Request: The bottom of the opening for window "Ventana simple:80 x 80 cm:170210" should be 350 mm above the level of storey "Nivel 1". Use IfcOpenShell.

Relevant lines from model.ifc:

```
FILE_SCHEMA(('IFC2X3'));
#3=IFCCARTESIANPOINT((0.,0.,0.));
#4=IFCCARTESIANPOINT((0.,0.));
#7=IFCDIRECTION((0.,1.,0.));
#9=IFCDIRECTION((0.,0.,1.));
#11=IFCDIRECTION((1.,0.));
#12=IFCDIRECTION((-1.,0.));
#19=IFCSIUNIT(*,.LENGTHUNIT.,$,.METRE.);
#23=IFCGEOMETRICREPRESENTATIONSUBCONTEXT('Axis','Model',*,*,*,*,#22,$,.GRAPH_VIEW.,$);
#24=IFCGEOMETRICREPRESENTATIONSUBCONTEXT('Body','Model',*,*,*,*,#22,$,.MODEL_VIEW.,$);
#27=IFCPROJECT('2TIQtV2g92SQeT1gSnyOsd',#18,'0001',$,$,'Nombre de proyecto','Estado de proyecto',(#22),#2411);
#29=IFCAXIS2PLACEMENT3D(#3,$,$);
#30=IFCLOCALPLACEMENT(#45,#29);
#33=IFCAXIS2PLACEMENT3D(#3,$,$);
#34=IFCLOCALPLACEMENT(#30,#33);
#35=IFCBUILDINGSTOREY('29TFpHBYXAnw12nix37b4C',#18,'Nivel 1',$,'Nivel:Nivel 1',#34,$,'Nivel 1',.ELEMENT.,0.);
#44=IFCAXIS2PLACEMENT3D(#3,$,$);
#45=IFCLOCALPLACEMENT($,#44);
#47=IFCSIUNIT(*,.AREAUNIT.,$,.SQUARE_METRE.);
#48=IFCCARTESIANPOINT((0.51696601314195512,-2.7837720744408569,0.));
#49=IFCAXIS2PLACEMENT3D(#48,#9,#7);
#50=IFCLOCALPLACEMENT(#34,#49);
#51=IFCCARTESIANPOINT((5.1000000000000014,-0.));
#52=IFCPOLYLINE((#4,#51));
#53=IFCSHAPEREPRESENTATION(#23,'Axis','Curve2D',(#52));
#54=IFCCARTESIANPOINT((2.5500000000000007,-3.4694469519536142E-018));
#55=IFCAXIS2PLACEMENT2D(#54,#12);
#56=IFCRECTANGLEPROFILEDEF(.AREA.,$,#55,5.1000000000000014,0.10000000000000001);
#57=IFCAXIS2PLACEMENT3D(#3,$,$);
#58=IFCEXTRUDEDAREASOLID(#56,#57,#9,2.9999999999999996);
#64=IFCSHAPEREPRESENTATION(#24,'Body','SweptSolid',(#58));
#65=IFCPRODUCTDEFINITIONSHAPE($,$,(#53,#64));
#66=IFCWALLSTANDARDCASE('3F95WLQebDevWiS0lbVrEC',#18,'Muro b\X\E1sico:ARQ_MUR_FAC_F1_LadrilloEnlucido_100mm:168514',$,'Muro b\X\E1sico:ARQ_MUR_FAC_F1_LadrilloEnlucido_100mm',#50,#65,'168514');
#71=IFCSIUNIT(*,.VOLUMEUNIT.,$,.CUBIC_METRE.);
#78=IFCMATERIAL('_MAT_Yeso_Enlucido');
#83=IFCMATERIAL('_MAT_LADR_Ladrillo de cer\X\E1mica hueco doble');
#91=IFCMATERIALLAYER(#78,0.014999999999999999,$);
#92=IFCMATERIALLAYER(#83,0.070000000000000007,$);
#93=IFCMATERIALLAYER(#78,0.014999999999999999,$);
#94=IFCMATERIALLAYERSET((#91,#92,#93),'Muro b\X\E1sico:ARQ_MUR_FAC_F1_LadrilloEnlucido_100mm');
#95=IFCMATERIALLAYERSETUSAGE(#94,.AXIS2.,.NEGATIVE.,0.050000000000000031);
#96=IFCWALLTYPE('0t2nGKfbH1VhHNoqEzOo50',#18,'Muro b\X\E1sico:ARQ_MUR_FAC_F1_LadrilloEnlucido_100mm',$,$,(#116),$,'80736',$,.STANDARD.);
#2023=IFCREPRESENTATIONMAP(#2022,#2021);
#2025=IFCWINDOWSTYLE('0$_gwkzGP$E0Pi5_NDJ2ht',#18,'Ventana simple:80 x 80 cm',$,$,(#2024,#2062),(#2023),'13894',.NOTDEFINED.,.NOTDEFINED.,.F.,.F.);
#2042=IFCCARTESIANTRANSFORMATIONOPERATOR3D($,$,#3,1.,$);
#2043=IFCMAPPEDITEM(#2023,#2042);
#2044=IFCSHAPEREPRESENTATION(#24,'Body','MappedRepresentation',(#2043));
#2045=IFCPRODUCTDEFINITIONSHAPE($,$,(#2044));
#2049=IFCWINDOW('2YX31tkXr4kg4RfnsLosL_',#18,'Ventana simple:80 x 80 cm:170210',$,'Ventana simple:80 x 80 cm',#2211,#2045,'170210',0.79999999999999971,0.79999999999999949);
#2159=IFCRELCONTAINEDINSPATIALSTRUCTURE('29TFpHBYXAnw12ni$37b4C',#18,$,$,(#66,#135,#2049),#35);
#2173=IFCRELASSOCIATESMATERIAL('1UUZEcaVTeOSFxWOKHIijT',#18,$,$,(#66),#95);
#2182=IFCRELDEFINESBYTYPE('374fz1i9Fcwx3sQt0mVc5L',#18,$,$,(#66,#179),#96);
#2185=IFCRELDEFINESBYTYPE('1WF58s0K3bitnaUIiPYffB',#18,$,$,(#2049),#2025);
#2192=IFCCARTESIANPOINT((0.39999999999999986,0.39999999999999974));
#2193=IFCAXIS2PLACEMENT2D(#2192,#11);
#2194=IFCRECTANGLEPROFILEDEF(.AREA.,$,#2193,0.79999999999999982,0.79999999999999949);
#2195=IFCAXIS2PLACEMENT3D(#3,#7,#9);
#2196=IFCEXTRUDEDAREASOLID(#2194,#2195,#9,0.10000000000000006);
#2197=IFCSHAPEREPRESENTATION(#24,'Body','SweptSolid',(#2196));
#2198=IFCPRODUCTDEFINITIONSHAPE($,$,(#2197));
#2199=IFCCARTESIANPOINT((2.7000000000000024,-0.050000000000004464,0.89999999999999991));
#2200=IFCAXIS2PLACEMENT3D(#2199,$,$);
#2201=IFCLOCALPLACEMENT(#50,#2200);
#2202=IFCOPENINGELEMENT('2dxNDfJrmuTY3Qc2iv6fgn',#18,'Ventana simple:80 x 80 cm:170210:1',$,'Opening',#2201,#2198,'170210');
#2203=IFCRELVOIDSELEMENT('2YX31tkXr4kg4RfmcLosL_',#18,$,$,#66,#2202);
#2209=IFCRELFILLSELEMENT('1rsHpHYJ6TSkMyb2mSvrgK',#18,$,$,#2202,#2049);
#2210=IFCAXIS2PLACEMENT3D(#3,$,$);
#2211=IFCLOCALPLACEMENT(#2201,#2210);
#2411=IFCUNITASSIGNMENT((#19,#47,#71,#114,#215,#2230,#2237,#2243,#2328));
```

```python
import numpy as np
import ifcopenshell
import ifcopenshell.api.geometry
import ifcopenshell.geom
import ifcopenshell.util.element
import ifcopenshell.util.placement
import ifcopenshell.util.shape
import ifcopenshell.util.unit

model = ifcopenshell.open("model.ifc")
unit_scale = ifcopenshell.util.unit.calculate_unit_scale(model)

window = model.by_guid("2YX31tkXr4kg4RfnsLosL_")
opening = window.FillsVoids[0].RelatingOpeningElement
storey = ifcopenshell.util.element.get_container(window, ifc_class="IfcBuildingStorey")
level = ifcopenshell.util.placement.get_local_placement(storey.ObjectPlacement)[2, 3]

# The opening's origin need not be at the sill, so measure its lowest point.
shape = ifcopenshell.geom.create_shape(ifcopenshell.geom.settings(), opening)
bottom = ifcopenshell.util.shape.get_shape_bottom_elevation(shape, shape.geometry) / unit_scale
dz = level + 0.35 - bottom

shift = np.array([0.0, 0.0, dz])
# The window is placed relative to its opening, so it follows when the opening moves.
matrix = ifcopenshell.util.placement.get_local_placement(opening.ObjectPlacement)
matrix[:3, 3] += shift
ifcopenshell.api.geometry.edit_object_placement(
    model, product=opening, matrix=matrix, is_si=False, should_transform_children=True
)

print(f"moved by {dz * unit_scale:+.3f} m")

model.write("model_rev.ifc")
```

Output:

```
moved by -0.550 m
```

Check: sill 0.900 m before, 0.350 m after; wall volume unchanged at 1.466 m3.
